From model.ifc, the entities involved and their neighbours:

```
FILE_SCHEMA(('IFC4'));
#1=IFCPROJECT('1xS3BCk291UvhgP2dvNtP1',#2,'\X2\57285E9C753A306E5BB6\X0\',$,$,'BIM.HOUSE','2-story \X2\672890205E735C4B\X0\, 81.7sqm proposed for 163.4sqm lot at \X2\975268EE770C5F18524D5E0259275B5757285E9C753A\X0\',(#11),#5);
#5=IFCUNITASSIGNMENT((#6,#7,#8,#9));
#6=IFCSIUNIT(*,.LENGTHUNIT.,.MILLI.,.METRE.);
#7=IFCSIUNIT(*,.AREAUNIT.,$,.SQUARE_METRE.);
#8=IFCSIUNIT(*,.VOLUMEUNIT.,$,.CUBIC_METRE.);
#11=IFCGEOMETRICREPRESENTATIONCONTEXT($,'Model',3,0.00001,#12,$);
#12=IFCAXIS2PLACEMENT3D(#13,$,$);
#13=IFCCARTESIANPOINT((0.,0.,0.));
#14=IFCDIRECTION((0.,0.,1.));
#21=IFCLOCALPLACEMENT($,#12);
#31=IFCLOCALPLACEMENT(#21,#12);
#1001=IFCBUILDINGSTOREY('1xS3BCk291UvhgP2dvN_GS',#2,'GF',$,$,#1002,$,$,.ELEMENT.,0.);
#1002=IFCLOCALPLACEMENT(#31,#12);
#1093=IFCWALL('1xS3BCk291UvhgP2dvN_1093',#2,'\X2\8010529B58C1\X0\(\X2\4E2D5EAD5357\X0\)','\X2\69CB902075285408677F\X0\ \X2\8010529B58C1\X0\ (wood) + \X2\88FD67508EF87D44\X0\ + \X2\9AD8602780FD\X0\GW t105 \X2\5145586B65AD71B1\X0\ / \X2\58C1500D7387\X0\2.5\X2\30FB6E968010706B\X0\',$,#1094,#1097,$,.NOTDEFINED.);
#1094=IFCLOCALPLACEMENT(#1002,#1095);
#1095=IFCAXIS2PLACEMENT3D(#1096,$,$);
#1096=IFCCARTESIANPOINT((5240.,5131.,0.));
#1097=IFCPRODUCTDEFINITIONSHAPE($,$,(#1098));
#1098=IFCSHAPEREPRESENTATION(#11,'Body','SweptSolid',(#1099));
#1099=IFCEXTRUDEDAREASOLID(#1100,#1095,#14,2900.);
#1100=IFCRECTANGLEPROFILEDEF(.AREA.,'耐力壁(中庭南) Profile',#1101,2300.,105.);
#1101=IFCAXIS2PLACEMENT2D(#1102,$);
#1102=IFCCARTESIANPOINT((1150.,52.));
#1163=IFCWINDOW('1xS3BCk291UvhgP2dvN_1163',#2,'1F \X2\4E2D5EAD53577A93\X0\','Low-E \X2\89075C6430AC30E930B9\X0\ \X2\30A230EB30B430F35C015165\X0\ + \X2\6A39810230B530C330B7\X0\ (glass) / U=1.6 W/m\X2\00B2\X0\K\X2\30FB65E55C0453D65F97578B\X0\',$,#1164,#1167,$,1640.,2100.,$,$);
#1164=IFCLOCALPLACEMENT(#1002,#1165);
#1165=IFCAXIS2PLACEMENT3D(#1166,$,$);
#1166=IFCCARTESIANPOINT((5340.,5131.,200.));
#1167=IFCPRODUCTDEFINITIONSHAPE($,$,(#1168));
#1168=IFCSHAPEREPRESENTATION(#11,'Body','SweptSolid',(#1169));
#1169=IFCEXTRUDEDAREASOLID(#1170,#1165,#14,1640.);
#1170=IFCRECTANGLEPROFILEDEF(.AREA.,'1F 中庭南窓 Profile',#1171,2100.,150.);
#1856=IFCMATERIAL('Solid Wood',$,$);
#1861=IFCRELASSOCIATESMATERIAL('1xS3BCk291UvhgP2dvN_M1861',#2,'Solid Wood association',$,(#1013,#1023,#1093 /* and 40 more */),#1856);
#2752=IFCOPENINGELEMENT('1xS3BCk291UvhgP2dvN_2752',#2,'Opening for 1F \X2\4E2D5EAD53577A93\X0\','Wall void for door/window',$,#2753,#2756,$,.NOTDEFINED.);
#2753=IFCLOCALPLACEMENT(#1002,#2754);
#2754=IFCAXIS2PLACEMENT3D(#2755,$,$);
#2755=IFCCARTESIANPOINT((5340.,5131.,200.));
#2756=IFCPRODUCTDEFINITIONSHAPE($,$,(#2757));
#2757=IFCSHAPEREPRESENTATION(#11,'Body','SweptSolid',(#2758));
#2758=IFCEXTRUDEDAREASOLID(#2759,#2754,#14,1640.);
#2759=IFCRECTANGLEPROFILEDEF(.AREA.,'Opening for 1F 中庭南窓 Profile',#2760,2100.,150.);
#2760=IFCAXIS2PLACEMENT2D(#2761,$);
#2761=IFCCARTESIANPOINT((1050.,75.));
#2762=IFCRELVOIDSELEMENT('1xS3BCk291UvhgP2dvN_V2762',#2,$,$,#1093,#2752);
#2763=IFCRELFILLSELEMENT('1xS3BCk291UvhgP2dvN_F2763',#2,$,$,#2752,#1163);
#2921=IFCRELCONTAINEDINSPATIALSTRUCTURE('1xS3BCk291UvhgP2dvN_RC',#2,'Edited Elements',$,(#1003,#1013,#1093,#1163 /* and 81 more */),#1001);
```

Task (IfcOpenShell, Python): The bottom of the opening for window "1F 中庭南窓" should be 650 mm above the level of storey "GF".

```python
import numpy as np
import ifcopenshell
import ifcopenshell.api.geometry
import ifcopenshell.geom
import ifcopenshell.util.element
import ifcopenshell.util.placement
import ifcopenshell.util.shape
import ifcopenshell.util.unit

model = ifcopenshell.open("model.ifc")
unit_scale = ifcopenshell.util.unit.calculate_unit_scale(model)

window = model.by_guid("1xS3BCk291UvhgP2dvN_1163")
opening = window.FillsVoids[0].RelatingOpeningElement
storey = ifcopenshell.util.element.get_container(window, ifc_class="IfcBuildingStorey")
level = ifcopenshell.util.placement.get_local_placement(storey.ObjectPlacement)[2, 3]

# The opening's origin need not be at the sill, so measure its lowest point.
shape = ifcopenshell.geom.create_shape(ifcopenshell.geom.settings(), opening)
bottom = ifcopenshell.util.shape.get_shape_bottom_elevation(shape, shape.geometry) / unit_scale
dz = level + 0.65 / unit_scale - bottom

shift = np.array([0.0, 0.0, dz])
# The window is not placed relative to its opening, so move both.
for product in (opening, window):
    matrix = ifcopenshell.util.placement.get_local_placement(product.ObjectPlacement)
    matrix[:3, 3] += shift
    ifcopenshell.api.geometry.edit_object_placement(model, product=product, matrix=matrix, is_si=False)

print(f"moved by {dz * unit_scale:+.3f} m")

model.write("model_updated.ifc")
```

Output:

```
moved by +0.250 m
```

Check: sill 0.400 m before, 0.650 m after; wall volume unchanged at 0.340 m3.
